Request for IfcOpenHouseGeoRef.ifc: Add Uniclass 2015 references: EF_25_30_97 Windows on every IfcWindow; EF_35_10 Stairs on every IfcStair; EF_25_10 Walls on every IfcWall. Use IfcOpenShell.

First a look at what the model holds.

```python
import ifcopenshell

model = ifcopenshell.open("IfcOpenHouseGeoRef.ifc")
print(model.schema)
print("classifications:", [c.Name for c in model.by_type("IfcClassification")])
for ifc_class in ("IfcDoor", "IfcRoof", "IfcStair", "IfcWall", "IfcWindow"):
    print(ifc_class, len(model.by_type(ifc_class)))
```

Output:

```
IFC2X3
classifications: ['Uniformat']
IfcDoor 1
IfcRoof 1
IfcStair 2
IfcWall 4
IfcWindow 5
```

```python
import ifcopenshell
import ifcopenshell.api.classification

model = ifcopenshell.open("IfcOpenHouseGeoRef.ifc")

# IFC2X3 requires Source and Edition and has no link from the project to the system.
system = model.create_entity("IfcClassification", Source="NBS", Edition="2015", Name="Uniclass 2015")

codes = {
    "IfcWindow": ("EF_25_30_97", "Windows"),
    "IfcStair": ("EF_35_10", "Stairs"),
    "IfcWall": ("EF_25_10", "Walls"),
}
for ifc_class, (code, name) in codes.items():
    products = model.by_type(ifc_class)
    ifcopenshell.api.classification.add_reference(
        model, products=products, classification=system, identification=code, name=name
    )
    print(code, len(products))

model.write("IfcOpenHouseGeoRef_edited.ifc")
```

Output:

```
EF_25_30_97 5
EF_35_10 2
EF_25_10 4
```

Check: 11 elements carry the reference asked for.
